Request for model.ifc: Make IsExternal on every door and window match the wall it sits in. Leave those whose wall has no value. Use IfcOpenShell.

First a look at what the model holds.

```python
import ifcopenshell
import ifcopenshell.util.element

model = ifcopenshell.open("model.ifc")
print(model.schema)
seen = {}
for e in model.by_type("IfcDoor") + model.by_type("IfcWindow"):
    if not e.FillsVoids:
        continue
    host = e.FillsVoids[0].RelatingOpeningElement.VoidsElements[0].RelatingBuildingElement
    own = ifcopenshell.util.element.get_pset(e, f"Pset_{e.is_a()[3:].removesuffix('StandardCase')}Common", "IsExternal")
    wall = ifcopenshell.util.element.get_pset(host, "Pset_WallCommon", "IsExternal")
    seen[e.is_a(), own, wall] = seen.get((e.is_a(), own, wall), 0) + 1
for (cls, own, wall), count in sorted(seen.items(), key=str):
    print(count, cls, "IsExternal:", own, "| host wall:", wall)
```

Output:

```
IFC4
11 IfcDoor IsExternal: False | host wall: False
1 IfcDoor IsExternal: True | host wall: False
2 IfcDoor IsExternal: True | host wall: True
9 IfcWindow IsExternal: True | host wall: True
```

```python
import ifcopenshell
import ifcopenshell.api.pset
import ifcopenshell.util.element

model = ifcopenshell.open("model.ifc")

count = 0
for ifc_class, pset_name in (("IfcDoor", "Pset_DoorCommon"), ("IfcWindow", "Pset_WindowCommon")):
    for e in model.by_type(ifc_class):
        if not e.FillsVoids:
            continue
        host = e.FillsVoids[0].RelatingOpeningElement.VoidsElements[0].RelatingBuildingElement
        external = ifcopenshell.util.element.get_pset(host, "Pset_WallCommon", "IsExternal")
        if external is None or ifcopenshell.util.element.get_pset(e, pset_name, "IsExternal") == external:
            continue
        pset = ifcopenshell.api.pset.add_pset(model, product=e, name=pset_name)
        ifcopenshell.api.pset.edit_pset(model, pset=pset, properties={"IsExternal": external})
        count += 1

print(count, "updated")

model.write("model-out.ifc")
```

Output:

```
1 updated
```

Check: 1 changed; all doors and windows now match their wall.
